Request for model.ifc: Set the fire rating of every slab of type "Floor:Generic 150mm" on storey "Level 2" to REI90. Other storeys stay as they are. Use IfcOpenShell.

First a look at what the model holds.

```python
import ifcopenshell
import ifcopenshell.util.element

model = ifcopenshell.open("model.ifc")
print(model.schema)
storey = next(s for s in model.by_type("IfcBuildingStorey") if s.Name == "Level 2")
slabs = [e for e in ifcopenshell.util.element.get_decomposition(storey) if e.is_a("IfcSlab")]
seen = {}
for e in slabs:
    element_type = ifcopenshell.util.element.get_type(e)
    key = (element_type.Name if element_type != e and element_type else None, ifcopenshell.util.element.get_pset(e, "Pset_SlabCommon", "FireRating"))
    seen[key] = seen.get(key, 0) + 1
for (name, value), count in sorted(seen.items(), key=str):
    print(count, "x", name, "|", value)
```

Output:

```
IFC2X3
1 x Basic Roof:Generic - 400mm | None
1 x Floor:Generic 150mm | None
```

```python
import ifcopenshell
import ifcopenshell.api.pset
import ifcopenshell.util.element

model = ifcopenshell.open("model.ifc")

storey = next(s for s in model.by_type("IfcBuildingStorey") if s.Name == "Level 2")
slabs = [e for e in ifcopenshell.util.element.get_decomposition(storey) if e.is_a("IfcSlab")]

count = 0
for e in slabs:
    element_type = ifcopenshell.util.element.get_type(e)
    if element_type in (None, e) or element_type.Name != "Floor:Generic 150mm":
        continue
    # add_pset returns the element's existing set when there is one.
    pset = ifcopenshell.api.pset.add_pset(model, product=e, name="Pset_SlabCommon")
    ifcopenshell.api.pset.edit_pset(model, pset=pset, properties={"FireRating": "REI90"})
    count += 1

print(count, "slabs updated")

model.write("model_edited.ifc")
```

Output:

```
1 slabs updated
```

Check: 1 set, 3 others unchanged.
